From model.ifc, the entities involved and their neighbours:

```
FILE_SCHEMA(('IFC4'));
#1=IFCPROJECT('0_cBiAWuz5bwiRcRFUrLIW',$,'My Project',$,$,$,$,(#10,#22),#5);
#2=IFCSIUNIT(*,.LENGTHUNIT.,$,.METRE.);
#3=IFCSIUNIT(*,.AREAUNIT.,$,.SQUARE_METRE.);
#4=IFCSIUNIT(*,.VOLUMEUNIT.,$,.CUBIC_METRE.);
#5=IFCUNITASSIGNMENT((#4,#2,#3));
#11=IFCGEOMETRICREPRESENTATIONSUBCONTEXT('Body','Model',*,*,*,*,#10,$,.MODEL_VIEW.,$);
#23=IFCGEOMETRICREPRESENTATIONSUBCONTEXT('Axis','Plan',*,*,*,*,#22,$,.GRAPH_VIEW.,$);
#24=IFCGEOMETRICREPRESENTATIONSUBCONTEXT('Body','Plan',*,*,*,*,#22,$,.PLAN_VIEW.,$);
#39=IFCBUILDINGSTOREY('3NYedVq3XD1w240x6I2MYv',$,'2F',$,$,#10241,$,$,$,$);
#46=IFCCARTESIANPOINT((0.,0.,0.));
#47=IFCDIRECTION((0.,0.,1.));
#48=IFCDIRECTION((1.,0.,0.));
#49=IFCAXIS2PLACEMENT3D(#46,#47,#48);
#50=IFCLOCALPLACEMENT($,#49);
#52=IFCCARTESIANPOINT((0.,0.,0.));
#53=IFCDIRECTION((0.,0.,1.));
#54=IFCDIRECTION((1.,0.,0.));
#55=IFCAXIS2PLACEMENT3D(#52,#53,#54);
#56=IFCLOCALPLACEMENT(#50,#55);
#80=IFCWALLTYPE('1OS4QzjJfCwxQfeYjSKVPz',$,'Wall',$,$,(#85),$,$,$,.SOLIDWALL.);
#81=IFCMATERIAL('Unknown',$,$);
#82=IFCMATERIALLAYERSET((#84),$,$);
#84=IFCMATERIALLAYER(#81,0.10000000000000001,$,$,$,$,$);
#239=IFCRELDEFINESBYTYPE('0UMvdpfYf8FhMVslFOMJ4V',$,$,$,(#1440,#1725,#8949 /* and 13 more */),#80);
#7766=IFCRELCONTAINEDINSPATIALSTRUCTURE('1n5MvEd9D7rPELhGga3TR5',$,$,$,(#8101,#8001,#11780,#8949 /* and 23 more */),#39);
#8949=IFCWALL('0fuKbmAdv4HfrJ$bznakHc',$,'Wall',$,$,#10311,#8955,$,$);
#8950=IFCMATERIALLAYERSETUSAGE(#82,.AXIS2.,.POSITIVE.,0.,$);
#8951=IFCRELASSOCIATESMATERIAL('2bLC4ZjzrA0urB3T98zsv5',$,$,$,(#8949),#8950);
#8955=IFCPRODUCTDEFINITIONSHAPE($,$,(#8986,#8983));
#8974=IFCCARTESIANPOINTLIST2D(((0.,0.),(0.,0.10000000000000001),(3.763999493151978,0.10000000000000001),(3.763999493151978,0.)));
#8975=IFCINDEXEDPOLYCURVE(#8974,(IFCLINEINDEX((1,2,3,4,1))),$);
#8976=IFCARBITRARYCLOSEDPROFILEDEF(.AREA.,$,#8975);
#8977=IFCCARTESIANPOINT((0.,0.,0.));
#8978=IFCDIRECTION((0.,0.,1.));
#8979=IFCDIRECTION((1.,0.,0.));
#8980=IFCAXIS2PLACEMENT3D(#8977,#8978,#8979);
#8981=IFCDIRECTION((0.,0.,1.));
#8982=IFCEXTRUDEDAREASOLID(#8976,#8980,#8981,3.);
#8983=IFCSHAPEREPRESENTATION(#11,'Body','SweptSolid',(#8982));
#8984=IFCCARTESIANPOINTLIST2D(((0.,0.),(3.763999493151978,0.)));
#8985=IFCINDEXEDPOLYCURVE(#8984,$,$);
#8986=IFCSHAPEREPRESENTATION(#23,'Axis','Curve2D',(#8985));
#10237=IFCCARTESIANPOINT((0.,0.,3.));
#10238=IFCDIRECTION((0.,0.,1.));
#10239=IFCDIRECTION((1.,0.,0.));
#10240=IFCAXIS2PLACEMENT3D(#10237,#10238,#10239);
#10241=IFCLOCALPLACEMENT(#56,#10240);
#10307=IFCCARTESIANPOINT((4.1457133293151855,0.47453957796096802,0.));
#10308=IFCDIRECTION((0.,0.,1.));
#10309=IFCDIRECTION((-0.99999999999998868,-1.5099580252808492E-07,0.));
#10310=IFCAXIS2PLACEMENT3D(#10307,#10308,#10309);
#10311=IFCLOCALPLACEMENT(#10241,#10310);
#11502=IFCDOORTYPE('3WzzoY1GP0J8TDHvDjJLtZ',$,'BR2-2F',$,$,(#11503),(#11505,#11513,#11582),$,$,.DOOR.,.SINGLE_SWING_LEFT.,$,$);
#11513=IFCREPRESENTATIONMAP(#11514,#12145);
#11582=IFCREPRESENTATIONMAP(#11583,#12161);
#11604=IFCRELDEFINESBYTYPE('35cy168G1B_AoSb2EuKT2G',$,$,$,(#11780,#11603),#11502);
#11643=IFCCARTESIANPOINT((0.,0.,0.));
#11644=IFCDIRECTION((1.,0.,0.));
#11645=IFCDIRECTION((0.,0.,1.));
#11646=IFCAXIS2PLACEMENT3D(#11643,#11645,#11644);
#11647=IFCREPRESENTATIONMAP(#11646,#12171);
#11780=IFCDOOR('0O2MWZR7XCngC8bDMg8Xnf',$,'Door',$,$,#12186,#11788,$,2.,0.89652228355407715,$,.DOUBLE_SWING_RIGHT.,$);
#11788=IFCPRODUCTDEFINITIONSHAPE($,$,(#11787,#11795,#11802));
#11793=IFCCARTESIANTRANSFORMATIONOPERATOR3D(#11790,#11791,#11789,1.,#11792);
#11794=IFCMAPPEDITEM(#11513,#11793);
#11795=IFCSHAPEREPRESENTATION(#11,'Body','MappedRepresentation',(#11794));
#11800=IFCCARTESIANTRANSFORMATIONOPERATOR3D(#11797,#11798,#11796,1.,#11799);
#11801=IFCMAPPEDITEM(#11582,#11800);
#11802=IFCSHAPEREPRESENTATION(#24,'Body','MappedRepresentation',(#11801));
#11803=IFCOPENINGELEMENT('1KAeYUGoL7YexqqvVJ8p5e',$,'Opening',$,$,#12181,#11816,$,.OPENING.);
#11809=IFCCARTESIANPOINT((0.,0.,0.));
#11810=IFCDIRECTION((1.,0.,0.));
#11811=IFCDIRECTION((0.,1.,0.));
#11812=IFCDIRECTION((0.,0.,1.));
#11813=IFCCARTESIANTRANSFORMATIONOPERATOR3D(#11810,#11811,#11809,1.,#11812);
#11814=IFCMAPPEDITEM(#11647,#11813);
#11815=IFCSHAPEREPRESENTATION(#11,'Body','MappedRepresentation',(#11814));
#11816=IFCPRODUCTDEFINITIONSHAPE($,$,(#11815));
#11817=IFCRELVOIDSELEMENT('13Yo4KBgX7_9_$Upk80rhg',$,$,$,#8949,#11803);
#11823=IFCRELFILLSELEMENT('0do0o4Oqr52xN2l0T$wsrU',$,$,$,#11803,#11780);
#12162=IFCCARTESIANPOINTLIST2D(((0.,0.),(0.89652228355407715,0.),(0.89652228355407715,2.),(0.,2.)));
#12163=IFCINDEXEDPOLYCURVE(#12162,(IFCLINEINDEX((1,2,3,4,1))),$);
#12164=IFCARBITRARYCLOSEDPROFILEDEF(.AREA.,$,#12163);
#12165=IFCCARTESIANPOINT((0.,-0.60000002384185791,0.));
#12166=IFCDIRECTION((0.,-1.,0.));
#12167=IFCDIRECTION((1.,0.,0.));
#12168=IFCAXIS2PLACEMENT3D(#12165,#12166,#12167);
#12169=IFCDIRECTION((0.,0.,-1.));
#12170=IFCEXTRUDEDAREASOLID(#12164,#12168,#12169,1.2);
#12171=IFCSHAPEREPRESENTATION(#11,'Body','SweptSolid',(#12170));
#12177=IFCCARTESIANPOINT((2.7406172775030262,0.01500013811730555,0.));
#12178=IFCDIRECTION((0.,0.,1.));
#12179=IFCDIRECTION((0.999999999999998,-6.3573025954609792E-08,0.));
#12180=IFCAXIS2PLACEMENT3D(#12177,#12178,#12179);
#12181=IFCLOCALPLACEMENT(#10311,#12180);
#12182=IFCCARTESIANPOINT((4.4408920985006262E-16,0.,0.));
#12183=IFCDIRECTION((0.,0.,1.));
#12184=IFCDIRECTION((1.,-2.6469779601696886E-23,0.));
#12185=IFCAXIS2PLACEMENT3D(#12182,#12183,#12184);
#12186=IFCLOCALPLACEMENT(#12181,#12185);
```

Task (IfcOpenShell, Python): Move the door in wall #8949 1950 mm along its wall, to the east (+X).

```python
import ifcopenshell
import ifcopenshell.api.geometry
import ifcopenshell.util.placement
import ifcopenshell.util.unit

model = ifcopenshell.open("model.ifc")
unit_scale = ifcopenshell.util.unit.calculate_unit_scale(model)

door = model.by_guid("0O2MWZR7XCngC8bDMg8Xnf")
opening = door.FillsVoids[0].RelatingOpeningElement
wall = opening.VoidsElements[0].RelatingBuildingElement

wall_matrix = ifcopenshell.util.placement.get_local_placement(wall.ObjectPlacement)
shift = wall_matrix[:3, 0] * -1.95 / unit_scale
before = ifcopenshell.util.placement.get_local_placement(door.ObjectPlacement)[:3, 3].copy()

# The door is placed relative to its opening, so it follows when the opening moves.
matrix = ifcopenshell.util.placement.get_local_placement(opening.ObjectPlacement)
matrix[:3, 3] += shift
ifcopenshell.api.geometry.edit_object_placement(
    model, product=opening, matrix=matrix, is_si=False, should_transform_children=True
)

after = ifcopenshell.util.placement.get_local_placement(door.ObjectPlacement)[:3, 3]
print("door moved by", (after - before).round(3) + 0.0)

model.write("model_edited.ifc")
```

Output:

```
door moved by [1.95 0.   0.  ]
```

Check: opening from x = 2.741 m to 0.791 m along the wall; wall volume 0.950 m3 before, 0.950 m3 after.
